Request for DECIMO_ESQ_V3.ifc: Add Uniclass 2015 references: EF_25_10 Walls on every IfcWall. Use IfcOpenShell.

First a look at what the model holds.

```python
import ifcopenshell

model = ifcopenshell.open("DECIMO_ESQ_V3.ifc")
print(model.schema)
print("classifications:", [c.Name for c in model.by_type("IfcClassification")])
for ifc_class in ("IfcDoor", "IfcRoof", "IfcStair", "IfcWall", "IfcWindow"):
    print(ifc_class, len(model.by_type(ifc_class)))
```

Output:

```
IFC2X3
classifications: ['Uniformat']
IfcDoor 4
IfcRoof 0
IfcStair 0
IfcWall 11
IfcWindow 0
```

```python
import ifcopenshell
import ifcopenshell.api.classification

model = ifcopenshell.open("DECIMO_ESQ_V3.ifc")

# IFC2X3 requires Source and Edition and has no link from the project to the system.
system = model.create_entity("IfcClassification", Source="NBS", Edition="2015", Name="Uniclass 2015")

codes = {
    "IfcWall": ("EF_25_10", "Walls"),
}
for ifc_class, (code, name) in codes.items():
    products = model.by_type(ifc_class)
    ifcopenshell.api.classification.add_reference(
        model, products=products, classification=system, identification=code, name=name
    )
    print(code, len(products))

model.write("DECIMO_ESQ_V3-out.ifc")
```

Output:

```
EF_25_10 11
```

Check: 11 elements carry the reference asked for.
